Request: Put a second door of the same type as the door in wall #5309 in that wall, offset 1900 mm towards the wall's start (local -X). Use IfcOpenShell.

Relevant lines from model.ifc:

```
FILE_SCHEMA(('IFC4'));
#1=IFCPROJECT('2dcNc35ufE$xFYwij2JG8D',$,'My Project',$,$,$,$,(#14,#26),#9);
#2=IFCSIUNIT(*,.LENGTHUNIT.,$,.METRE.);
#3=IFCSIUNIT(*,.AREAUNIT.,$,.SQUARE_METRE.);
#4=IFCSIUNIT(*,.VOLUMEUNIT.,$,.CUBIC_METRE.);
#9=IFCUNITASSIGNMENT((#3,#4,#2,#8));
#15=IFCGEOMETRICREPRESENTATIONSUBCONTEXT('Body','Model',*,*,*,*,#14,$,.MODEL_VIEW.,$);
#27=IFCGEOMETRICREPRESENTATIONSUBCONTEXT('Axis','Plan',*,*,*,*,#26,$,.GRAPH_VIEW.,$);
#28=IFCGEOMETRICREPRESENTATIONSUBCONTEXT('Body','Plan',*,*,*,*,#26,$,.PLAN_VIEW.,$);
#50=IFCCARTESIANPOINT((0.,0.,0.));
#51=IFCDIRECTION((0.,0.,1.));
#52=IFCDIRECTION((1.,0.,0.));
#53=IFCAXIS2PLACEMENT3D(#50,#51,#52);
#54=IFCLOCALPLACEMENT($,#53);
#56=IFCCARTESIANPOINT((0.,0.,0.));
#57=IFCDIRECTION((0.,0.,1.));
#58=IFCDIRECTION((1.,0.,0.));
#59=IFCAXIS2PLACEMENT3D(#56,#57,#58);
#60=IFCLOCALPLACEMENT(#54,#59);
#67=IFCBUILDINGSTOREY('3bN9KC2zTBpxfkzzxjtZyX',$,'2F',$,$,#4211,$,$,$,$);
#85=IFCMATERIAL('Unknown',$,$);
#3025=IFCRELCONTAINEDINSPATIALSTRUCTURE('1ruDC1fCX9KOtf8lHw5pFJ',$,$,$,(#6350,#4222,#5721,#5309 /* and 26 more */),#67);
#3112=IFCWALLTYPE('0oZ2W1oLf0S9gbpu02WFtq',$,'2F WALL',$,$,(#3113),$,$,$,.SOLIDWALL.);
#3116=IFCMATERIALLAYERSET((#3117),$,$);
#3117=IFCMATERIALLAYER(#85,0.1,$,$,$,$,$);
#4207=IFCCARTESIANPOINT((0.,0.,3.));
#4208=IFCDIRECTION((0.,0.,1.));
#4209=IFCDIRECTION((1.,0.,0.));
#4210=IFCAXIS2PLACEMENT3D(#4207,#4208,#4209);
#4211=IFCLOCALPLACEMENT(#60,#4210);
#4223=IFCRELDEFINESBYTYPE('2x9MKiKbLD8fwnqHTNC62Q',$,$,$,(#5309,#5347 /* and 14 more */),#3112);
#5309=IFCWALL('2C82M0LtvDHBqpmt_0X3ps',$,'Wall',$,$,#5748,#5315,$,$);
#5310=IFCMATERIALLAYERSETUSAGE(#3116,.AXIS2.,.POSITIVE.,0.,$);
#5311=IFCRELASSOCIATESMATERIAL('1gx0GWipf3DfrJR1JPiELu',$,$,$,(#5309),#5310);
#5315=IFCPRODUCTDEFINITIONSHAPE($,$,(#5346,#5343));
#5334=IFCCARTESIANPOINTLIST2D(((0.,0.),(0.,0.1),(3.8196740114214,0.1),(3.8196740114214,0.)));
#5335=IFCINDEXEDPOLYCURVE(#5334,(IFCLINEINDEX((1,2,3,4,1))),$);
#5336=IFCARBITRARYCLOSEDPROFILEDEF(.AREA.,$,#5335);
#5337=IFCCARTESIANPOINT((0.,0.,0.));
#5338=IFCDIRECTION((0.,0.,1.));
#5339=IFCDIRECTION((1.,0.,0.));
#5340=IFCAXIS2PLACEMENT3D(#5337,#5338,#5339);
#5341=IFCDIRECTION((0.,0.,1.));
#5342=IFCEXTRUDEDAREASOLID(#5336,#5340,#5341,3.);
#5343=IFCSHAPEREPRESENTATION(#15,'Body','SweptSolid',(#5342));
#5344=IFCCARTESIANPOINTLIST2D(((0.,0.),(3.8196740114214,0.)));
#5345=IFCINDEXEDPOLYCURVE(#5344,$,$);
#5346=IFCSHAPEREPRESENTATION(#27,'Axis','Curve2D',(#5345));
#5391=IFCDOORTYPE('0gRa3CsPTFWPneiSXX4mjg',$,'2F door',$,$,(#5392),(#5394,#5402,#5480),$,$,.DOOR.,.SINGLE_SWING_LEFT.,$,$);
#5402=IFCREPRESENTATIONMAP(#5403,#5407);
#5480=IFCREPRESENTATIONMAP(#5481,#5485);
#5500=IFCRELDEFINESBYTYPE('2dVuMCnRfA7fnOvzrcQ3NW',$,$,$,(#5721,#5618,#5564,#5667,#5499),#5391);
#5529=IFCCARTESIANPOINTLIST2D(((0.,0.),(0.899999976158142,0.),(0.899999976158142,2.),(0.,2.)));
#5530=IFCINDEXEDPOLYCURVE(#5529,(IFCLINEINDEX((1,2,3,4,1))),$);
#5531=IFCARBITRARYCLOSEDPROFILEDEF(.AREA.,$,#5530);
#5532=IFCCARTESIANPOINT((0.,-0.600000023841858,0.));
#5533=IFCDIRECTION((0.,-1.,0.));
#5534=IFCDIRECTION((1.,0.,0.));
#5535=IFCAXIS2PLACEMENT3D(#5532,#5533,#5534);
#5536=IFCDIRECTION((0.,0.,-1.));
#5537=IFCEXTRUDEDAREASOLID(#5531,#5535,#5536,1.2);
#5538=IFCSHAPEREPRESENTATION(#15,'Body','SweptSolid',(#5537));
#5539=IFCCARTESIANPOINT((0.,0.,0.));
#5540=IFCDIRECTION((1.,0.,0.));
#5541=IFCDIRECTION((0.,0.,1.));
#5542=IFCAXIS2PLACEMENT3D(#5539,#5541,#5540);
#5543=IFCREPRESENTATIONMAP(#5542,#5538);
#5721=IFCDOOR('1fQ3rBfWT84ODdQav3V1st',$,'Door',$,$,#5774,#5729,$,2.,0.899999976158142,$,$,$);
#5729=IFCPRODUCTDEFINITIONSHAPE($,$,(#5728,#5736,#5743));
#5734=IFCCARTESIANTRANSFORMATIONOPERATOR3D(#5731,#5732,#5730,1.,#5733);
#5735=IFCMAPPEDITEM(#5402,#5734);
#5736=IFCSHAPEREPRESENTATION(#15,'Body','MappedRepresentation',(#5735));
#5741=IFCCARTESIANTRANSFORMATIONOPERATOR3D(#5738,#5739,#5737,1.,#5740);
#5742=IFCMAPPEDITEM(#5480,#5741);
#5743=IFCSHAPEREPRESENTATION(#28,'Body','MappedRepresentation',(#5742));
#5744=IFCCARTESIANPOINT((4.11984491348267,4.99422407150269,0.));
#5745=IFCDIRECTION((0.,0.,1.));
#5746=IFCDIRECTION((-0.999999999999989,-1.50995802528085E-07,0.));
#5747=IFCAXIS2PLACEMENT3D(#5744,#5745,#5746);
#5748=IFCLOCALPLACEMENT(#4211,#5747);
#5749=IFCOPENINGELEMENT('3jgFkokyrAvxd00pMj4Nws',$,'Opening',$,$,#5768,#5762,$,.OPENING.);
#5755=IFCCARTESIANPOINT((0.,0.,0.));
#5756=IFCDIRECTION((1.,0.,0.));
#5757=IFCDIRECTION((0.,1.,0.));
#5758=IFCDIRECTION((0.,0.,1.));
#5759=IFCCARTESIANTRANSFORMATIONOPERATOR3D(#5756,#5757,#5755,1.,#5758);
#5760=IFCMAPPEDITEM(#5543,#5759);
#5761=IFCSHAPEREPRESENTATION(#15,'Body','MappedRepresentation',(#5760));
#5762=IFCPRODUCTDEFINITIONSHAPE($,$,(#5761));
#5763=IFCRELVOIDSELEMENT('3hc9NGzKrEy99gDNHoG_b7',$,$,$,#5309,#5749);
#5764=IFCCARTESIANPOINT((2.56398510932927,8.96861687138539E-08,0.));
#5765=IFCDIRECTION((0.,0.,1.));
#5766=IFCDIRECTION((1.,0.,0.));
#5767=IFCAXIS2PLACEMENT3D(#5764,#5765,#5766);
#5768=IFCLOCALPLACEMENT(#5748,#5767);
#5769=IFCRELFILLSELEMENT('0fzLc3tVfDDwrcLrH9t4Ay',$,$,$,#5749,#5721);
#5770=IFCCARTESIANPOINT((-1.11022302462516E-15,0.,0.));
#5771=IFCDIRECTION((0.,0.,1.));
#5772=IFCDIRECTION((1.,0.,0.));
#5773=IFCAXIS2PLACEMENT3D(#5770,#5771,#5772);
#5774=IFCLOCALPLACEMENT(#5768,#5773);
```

```python
import ifcopenshell
import ifcopenshell.api.feature
import ifcopenshell.api.geometry
import ifcopenshell.api.root
import ifcopenshell.geom
import ifcopenshell.util.element
import ifcopenshell.util.placement
import ifcopenshell.util.shape
import ifcopenshell.util.unit

model = ifcopenshell.open("model.ifc")
unit_scale = ifcopenshell.util.unit.calculate_unit_scale(model)
settings = ifcopenshell.geom.settings()


def volume(element):
    """Net volume in cubic metres, openings subtracted."""
    shape = ifcopenshell.geom.create_shape(settings, element)
    return ifcopenshell.util.shape.get_volume(shape.geometry)


door = model.by_id(5721)
opening = door.FillsVoids[0].RelatingOpeningElement
wall = opening.VoidsElements[0].RelatingBuildingElement
before = volume(wall)
shift = ifcopenshell.util.placement.get_local_placement(wall.ObjectPlacement)[:3, 0] * -1.9 / unit_scale

# copy_class copies the void relationship, type, container and properties, but no geometry.
new_opening = ifcopenshell.api.root.copy_class(model, product=opening)
new_opening.Representation = ifcopenshell.util.element.copy_deep(
    model, opening.Representation, exclude=["IfcGeometricRepresentationContext", "IfcRepresentationMap"]
)
new_door = ifcopenshell.api.root.copy_class(model, product=door)
new_door.Representation = ifcopenshell.util.element.copy_deep(
    model, door.Representation, exclude=["IfcGeometricRepresentationContext", "IfcRepresentationMap"]
)
ifcopenshell.api.feature.add_filling(model, opening=new_opening, element=new_door)

for old, new in ((opening, new_opening), (door, new_door)):
    matrix = ifcopenshell.util.placement.get_local_placement(old.ObjectPlacement)
    matrix[:3, 3] += shift
    ifcopenshell.api.geometry.edit_object_placement(model, product=new, matrix=matrix, is_si=False)

after = volume(wall)

print(f"wall volume {before:.3f} -> {after:.3f} m3")

model.write("model_v2.ifc")
```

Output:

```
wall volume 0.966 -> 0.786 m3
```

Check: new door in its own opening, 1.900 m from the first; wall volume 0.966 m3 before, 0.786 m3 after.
